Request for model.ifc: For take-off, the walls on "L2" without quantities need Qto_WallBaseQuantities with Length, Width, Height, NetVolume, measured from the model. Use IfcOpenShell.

First a look at what the model holds.

```python
import ifcopenshell
import ifcopenshell.util.element
import ifcopenshell.util.unit

model = ifcopenshell.open("model.ifc")
print(model.schema)
for unit_type in ("LENGTHUNIT", "AREAUNIT", "VOLUMEUNIT"):
    print(unit_type, ifcopenshell.util.unit.calculate_unit_scale(model, unit_type))
storey = next(s for s in model.by_type("IfcBuildingStorey") if s.Name == "L2")
walls = [e for e in ifcopenshell.util.element.get_decomposition(storey) if e.is_a("IfcWall")]
for e in sorted(walls, key=lambda e: e.id()):
    print(e.id(), e.is_a(), e.Name, list(ifcopenshell.util.element.get_psets(e, qtos_only=True)), sep=" | ")
```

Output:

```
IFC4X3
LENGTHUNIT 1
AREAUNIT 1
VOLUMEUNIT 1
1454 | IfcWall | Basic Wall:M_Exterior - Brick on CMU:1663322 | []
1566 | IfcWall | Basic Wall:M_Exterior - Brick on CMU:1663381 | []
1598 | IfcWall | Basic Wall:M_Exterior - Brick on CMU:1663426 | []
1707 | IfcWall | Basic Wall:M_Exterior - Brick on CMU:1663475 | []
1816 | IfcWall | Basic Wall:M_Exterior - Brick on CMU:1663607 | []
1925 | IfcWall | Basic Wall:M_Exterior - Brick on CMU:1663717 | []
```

```python
import ifcopenshell
import ifcopenshell.api.pset
import ifcopenshell.geom
import ifcopenshell.util.element
import ifcopenshell.util.shape
import ifcopenshell.util.unit

model = ifcopenshell.open("model.ifc")
unit_scale = ifcopenshell.util.unit.calculate_unit_scale(model)
volume_scale = ifcopenshell.util.unit.calculate_unit_scale(model, "VOLUMEUNIT")
settings = ifcopenshell.geom.settings()

storey = next(s for s in model.by_type("IfcBuildingStorey") if s.Name == "L2")
walls = [e for e in ifcopenshell.util.element.get_decomposition(storey) if e.is_a("IfcWall")]

for e in sorted(walls, key=lambda e: e.id()):
    if ifcopenshell.util.element.get_psets(e, qtos_only=True, should_inherit=False):
        continue
    # Geometry comes back in metres, in the element's own axes.
    shape = ifcopenshell.geom.create_shape(settings, e)
    values = {
        "Length": ifcopenshell.util.shape.get_x(shape.geometry) / unit_scale,
        "Width": ifcopenshell.util.shape.get_y(shape.geometry) / unit_scale,
        "Height": ifcopenshell.util.shape.get_z(shape.geometry) / unit_scale,
        "NetVolume": ifcopenshell.util.shape.get_volume(shape.geometry) / volume_scale,
    }
    qto = ifcopenshell.api.pset.add_qto(model, product=e, name="Qto_WallBaseQuantities")
    ifcopenshell.api.pset.edit_qto(model, qto=qto, properties=values)
    print(e.id(), {k: round(v, 3) for k, v in values.items()})

model.write("model_rev.ifc")
```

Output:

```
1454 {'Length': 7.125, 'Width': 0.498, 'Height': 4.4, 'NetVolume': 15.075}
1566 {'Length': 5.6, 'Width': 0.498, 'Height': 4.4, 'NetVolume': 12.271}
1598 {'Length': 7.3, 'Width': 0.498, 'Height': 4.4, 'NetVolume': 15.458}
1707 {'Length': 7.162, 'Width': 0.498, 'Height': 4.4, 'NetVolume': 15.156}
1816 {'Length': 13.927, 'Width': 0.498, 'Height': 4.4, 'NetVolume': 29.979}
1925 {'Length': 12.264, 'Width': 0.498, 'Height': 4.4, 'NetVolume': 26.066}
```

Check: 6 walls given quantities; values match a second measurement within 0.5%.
